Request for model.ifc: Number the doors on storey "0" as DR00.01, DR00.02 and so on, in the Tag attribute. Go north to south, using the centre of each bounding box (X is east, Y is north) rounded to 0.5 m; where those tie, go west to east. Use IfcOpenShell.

First a look at what the model holds.

```python
import ifcopenshell
import ifcopenshell.util.element
import ifcopenshell.util.placement

model = ifcopenshell.open("model.ifc")
print(model.schema)
storey = next(s for s in model.by_type("IfcBuildingStorey") if s.Name == "0")
doors = [e for e in ifcopenshell.util.element.get_decomposition(storey) if e.is_a("IfcDoor")]
for e in sorted(doors, key=lambda e: e.id()):
    origin = ifcopenshell.util.placement.get_local_placement(e.ObjectPlacement)[:3, 3]
    print(e.id(), e.Tag, e.Name, origin.round(2) + 0.0, sep=" | ")
```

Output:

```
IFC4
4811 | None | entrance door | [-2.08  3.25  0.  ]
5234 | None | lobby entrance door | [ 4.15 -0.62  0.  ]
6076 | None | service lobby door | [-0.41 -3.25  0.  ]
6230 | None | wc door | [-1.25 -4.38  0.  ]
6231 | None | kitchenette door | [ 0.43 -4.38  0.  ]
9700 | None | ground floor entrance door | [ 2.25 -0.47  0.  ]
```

```python
import ifcopenshell
import ifcopenshell.geom
import ifcopenshell.util.element
import ifcopenshell.util.shape

model = ifcopenshell.open("model.ifc")
settings = ifcopenshell.geom.settings()
settings.set("use-world-coords", True)


def centre(element):
    shape = ifcopenshell.geom.create_shape(settings, element)
    return ifcopenshell.util.shape.get_bbox_centroid(shape.geometry)


storey = next(s for s in model.by_type("IfcBuildingStorey") if s.Name == "0")
doors = [e for e in ifcopenshell.util.element.get_decomposition(storey) if e.is_a("IfcDoor")]

# Insertion points can sit at a corner or the storey origin, so sort by the geometry (in metres).
centres = {e: centre(e) for e in doors}
doors.sort(key=lambda e: (-round(centres[e][1] / 0.5), centres[e][0]))

for i, e in enumerate(doors, start=1):
    number = f"DR00.{i:02d}"
    e.Tag = number
    print(e.id(), number)

model.write("model_edited.ifc")
```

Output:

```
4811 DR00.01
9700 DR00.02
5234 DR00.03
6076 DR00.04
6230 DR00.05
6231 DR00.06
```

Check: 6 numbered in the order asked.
